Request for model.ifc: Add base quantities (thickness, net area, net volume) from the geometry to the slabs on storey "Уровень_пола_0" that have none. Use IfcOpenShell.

First a look at what the model holds.

```python
import ifcopenshell
import ifcopenshell.util.element
import ifcopenshell.util.unit

model = ifcopenshell.open("model.ifc")
print(model.schema)
for unit_type in ("LENGTHUNIT", "AREAUNIT", "VOLUMEUNIT"):
    print(unit_type, ifcopenshell.util.unit.calculate_unit_scale(model, unit_type))
storey = next(s for s in model.by_type("IfcBuildingStorey") if s.Name == "Уровень_пола_0")
slabs = [e for e in ifcopenshell.util.element.get_decomposition(storey) if e.is_a("IfcSlab")]
for e in sorted(slabs, key=lambda e: e.id()):
    print(e.id(), e.is_a(), e.Name, list(ifcopenshell.util.element.get_psets(e, qtos_only=True)), sep=" | ")
```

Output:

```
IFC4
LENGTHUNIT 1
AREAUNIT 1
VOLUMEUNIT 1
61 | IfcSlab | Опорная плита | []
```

```python
import ifcopenshell
import ifcopenshell.api.pset
import ifcopenshell.geom
import ifcopenshell.util.element
import ifcopenshell.util.shape
import ifcopenshell.util.unit

model = ifcopenshell.open("model.ifc")
unit_scale = ifcopenshell.util.unit.calculate_unit_scale(model)
area_scale = ifcopenshell.util.unit.calculate_unit_scale(model, "AREAUNIT")
volume_scale = ifcopenshell.util.unit.calculate_unit_scale(model, "VOLUMEUNIT")
settings = ifcopenshell.geom.settings()

storey = next(s for s in model.by_type("IfcBuildingStorey") if s.Name == "Уровень_пола_0")
slabs = [e for e in ifcopenshell.util.element.get_decomposition(storey) if e.is_a("IfcSlab")]

for e in sorted(slabs, key=lambda e: e.id()):
    if ifcopenshell.util.element.get_psets(e, qtos_only=True, should_inherit=False):
        continue
    # Geometry comes back in metres, in the element's own axes.
    shape = ifcopenshell.geom.create_shape(settings, e)
    values = {
        "Width": ifcopenshell.util.shape.get_z(shape.geometry) / unit_scale,
        "NetArea": ifcopenshell.util.shape.get_footprint_area(shape.geometry) / area_scale,
        "NetVolume": ifcopenshell.util.shape.get_volume(shape.geometry) / volume_scale,
    }
    qto = ifcopenshell.api.pset.add_qto(model, product=e, name="Qto_SlabBaseQuantities")
    ifcopenshell.api.pset.edit_qto(model, qto=qto, properties=values)
    print(e.id(), {k: round(v, 3) for k, v in values.items()})

model.write("model-out.ifc")
```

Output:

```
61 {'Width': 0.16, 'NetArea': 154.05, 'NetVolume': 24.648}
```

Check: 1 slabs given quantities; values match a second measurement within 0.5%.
